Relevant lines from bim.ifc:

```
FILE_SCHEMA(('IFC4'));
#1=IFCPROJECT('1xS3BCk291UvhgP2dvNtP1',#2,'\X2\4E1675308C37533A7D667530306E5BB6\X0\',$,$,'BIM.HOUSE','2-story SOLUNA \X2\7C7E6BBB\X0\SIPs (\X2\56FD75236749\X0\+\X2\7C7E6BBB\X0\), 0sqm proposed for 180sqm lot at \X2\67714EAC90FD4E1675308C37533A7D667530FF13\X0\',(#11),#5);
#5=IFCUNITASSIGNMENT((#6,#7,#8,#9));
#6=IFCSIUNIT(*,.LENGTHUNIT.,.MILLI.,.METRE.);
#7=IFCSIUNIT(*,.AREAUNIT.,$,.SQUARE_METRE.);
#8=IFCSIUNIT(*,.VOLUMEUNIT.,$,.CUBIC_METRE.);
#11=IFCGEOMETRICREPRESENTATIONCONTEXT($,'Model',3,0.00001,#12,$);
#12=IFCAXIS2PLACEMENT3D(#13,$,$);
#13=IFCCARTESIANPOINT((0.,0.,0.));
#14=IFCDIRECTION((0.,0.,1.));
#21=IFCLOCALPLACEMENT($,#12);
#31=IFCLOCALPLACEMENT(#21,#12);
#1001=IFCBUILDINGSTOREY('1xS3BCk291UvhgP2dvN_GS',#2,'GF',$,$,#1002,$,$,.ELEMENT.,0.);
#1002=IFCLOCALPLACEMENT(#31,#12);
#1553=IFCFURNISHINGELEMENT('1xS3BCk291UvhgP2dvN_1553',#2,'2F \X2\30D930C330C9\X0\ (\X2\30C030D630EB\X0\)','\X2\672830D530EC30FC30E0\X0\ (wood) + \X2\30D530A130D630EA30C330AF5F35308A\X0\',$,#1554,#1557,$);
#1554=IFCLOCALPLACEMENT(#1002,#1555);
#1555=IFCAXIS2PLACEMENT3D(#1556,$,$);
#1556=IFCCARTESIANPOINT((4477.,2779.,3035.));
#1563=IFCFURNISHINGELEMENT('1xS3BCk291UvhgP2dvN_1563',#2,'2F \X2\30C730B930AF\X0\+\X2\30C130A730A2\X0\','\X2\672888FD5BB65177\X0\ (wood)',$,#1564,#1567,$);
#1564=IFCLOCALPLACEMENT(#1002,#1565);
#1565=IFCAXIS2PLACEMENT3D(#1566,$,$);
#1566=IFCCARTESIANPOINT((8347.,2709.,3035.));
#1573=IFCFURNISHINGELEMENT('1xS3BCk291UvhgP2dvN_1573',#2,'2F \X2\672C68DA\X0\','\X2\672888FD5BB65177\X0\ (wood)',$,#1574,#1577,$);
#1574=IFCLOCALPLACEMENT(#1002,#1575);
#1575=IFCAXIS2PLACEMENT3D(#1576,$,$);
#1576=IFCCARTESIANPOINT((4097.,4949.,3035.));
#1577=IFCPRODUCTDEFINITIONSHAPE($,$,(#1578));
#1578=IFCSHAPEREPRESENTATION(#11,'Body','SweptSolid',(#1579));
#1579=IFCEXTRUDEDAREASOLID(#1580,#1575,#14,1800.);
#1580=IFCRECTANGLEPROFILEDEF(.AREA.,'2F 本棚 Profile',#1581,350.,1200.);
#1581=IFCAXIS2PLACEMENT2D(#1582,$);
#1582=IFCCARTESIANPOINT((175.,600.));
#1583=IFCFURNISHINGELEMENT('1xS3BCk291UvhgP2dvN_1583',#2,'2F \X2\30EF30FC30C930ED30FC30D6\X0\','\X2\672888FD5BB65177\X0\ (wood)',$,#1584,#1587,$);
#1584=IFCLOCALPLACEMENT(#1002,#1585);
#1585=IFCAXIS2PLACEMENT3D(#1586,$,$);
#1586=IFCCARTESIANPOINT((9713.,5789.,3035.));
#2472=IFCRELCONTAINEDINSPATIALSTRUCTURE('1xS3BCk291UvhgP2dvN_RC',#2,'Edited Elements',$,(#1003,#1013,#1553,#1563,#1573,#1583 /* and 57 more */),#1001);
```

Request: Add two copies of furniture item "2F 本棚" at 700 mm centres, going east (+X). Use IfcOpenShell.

```python
import numpy as np
import ifcopenshell
import ifcopenshell.api.geometry
import ifcopenshell.api.root
import ifcopenshell.util.element
import ifcopenshell.util.placement
import ifcopenshell.util.unit

model = ifcopenshell.open("bim.ifc")
unit_scale = ifcopenshell.util.unit.calculate_unit_scale(model)


def reuse_history(source, copy):
    """copy_class also copies each property set's owner history, people and application; keep the originals."""
    for rel in copy.IsDefinedBy:
        if rel.is_a("IfcRelDefinesByProperties") and (history := rel.RelatingPropertyDefinition.OwnerHistory):
            rel.RelatingPropertyDefinition.OwnerHistory = source.OwnerHistory
            ifcopenshell.util.element.remove_deep2(model, history)


source = model.by_id(1573)
base = ifcopenshell.util.placement.get_local_placement(source.ObjectPlacement)
step = np.array([1.0, 0.0, 0.0]) * 0.7 / unit_scale

for i in range(1, 3):
    copy = ifcopenshell.api.root.copy_class(model, product=source)
    copy.Representation = ifcopenshell.util.element.copy_deep(
        model, source.Representation, exclude=["IfcGeometricRepresentationContext", "IfcRepresentationMap"]
    )
    reuse_history(source, copy)
    matrix = base.copy()
    matrix[:3, 3] += i * step
    print("added at", matrix[:3, 3].round(3) + 0.0)
    ifcopenshell.api.geometry.edit_object_placement(model, product=copy, matrix=matrix, is_si=False)

model.write("bim_v2.ifc")
```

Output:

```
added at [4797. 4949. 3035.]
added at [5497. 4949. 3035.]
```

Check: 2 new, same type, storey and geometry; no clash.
